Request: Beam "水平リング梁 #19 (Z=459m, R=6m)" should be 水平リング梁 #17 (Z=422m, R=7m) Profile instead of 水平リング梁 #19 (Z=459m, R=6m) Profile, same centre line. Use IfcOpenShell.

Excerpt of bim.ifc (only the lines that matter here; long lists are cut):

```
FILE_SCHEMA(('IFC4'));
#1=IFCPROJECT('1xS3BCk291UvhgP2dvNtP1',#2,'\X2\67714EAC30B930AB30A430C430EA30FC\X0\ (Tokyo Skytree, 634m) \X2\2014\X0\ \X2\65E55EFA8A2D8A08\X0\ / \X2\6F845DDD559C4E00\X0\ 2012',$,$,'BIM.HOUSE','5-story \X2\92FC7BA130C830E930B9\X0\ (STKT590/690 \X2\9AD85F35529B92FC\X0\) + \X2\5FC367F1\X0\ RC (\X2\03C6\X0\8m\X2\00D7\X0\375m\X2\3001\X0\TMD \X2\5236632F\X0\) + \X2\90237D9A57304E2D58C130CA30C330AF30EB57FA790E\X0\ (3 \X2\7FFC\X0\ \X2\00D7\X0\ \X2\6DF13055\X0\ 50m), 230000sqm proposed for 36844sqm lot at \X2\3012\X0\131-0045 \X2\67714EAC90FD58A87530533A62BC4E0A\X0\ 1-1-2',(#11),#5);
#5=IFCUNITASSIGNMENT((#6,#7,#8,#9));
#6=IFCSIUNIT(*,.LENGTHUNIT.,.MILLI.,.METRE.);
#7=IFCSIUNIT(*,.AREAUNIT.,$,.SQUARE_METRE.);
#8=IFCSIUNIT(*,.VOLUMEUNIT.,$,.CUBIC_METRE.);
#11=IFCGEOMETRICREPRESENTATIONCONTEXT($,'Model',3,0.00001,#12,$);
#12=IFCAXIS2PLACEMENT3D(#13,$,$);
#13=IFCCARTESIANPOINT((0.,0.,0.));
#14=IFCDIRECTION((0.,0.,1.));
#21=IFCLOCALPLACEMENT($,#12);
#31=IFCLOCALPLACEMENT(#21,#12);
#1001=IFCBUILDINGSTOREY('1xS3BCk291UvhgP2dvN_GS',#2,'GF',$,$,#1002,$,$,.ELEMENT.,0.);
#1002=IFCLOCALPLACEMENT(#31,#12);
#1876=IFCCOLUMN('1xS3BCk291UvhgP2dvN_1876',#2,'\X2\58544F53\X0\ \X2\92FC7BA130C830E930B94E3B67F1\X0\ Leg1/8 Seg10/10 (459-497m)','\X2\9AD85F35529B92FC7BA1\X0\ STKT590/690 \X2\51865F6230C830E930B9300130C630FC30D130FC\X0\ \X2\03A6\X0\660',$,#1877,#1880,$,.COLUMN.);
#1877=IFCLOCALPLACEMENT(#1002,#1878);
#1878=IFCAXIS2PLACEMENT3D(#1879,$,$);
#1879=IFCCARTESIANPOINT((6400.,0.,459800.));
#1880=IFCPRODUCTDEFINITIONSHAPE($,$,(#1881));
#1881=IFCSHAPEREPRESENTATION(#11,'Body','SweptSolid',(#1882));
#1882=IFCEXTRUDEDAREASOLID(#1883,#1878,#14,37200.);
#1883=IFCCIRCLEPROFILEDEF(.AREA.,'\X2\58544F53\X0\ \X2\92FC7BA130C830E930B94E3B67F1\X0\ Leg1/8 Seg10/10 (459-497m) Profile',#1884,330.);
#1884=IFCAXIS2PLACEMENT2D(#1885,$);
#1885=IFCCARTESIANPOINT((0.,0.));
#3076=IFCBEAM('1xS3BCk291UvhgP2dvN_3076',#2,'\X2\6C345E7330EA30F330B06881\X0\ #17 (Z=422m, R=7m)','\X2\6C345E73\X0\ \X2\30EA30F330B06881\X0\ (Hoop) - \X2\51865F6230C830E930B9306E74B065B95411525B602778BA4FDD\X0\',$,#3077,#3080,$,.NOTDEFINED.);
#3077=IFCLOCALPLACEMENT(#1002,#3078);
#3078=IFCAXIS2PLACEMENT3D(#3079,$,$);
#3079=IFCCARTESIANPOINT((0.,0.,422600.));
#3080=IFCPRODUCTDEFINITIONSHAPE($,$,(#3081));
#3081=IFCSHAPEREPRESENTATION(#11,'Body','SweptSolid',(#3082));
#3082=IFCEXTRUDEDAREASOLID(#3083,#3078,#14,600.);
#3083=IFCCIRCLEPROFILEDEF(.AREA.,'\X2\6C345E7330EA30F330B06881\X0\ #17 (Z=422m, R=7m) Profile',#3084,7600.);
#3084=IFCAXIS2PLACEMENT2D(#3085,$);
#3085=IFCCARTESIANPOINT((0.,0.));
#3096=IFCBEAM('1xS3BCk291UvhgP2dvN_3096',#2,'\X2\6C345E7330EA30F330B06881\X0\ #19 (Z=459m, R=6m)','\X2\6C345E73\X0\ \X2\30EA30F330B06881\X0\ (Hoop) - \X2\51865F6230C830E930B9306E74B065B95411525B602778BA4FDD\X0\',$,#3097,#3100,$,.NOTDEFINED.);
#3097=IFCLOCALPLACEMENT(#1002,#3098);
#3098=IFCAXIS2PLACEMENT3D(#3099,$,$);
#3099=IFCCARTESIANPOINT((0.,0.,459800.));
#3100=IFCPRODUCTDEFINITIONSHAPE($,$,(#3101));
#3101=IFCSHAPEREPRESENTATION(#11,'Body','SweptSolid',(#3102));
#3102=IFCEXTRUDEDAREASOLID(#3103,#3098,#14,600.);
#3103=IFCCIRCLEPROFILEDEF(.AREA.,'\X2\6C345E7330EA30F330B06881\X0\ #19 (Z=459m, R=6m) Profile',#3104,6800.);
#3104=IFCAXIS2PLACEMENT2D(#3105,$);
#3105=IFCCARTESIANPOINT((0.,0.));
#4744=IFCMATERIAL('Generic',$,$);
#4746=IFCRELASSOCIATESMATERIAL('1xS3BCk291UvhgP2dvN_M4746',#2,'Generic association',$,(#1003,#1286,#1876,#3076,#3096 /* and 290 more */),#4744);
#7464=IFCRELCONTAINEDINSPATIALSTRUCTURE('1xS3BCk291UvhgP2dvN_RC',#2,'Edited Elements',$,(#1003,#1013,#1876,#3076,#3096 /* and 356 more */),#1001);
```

```python
import ifcopenshell
import ifcopenshell.util.element

model = ifcopenshell.open("bim.ifc")

member = model.by_guid("1xS3BCk291UvhgP2dvN_3096")
source = next(p for p in model.by_type("IfcCircleProfileDef") if p.ProfileName == "水平リング梁 #17 (Z=422m, R=7m) Profile")

body = next(r for r in member.Representation.Representations if r.RepresentationIdentifier == "Body")
solid = body.Items[0]
old_profile = solid.SweptArea

# Copy the section's sizes but keep this member's own profile position.
profile = ifcopenshell.util.element.copy(model, source)
profile.Position = old_profile.Position
solid.SweptArea = profile
if not model.get_total_inverses(old_profile):
    ifcopenshell.util.element.remove_deep2(model, old_profile)

print(solid.SweptArea)

model.write("bim_v2.ifc")
```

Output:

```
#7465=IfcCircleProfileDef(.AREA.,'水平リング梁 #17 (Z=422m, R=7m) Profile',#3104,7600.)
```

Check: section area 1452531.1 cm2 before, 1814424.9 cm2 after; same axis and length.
